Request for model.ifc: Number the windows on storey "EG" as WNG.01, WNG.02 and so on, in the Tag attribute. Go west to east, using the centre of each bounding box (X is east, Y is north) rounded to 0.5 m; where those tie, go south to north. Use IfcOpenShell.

First a look at what the model holds.

```python
import ifcopenshell
import ifcopenshell.util.element
import ifcopenshell.util.placement

model = ifcopenshell.open("model.ifc")
print(model.schema)
storey = next(s for s in model.by_type("IfcBuildingStorey") if s.Name == "EG")
windows = [e for e in ifcopenshell.util.element.get_decomposition(storey) if e.is_a("IfcWindow")]
for e in sorted(windows, key=lambda e: e.id()):
    origin = ifcopenshell.util.placement.get_local_placement(e.ObjectPlacement)[:3, 3]
    print(e.id(), e.Tag, e.Name, origin.round(2) + 0.0, sep=" | ")
```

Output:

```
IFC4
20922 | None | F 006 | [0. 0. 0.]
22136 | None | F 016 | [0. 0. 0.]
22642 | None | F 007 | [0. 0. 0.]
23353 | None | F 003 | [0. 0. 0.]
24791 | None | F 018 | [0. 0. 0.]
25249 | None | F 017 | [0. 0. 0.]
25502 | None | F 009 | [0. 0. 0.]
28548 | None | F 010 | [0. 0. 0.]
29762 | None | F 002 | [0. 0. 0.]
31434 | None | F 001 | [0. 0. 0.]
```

```python
import ifcopenshell
import ifcopenshell.geom
import ifcopenshell.util.element
import ifcopenshell.util.shape

model = ifcopenshell.open("model.ifc")
settings = ifcopenshell.geom.settings()
settings.set("use-world-coords", True)


def centre(element):
    shape = ifcopenshell.geom.create_shape(settings, element)
    return ifcopenshell.util.shape.get_bbox_centroid(shape.geometry)


storey = next(s for s in model.by_type("IfcBuildingStorey") if s.Name == "EG")
windows = [e for e in ifcopenshell.util.element.get_decomposition(storey) if e.is_a("IfcWindow")]

# Insertion points can sit at a corner or the storey origin, so sort by the geometry (in metres).
centres = {e: centre(e) for e in windows}
windows.sort(key=lambda e: (round(centres[e][0] / 0.5), centres[e][1]))

for i, e in enumerate(windows, start=1):
    number = f"WNG.{i:02d}"
    e.Tag = number
    print(e.id(), number)

model.write("model_rev.ifc")
```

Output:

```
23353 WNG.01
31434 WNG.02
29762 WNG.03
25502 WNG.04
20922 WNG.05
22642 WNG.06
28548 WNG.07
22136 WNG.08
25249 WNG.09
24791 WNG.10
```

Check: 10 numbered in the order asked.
